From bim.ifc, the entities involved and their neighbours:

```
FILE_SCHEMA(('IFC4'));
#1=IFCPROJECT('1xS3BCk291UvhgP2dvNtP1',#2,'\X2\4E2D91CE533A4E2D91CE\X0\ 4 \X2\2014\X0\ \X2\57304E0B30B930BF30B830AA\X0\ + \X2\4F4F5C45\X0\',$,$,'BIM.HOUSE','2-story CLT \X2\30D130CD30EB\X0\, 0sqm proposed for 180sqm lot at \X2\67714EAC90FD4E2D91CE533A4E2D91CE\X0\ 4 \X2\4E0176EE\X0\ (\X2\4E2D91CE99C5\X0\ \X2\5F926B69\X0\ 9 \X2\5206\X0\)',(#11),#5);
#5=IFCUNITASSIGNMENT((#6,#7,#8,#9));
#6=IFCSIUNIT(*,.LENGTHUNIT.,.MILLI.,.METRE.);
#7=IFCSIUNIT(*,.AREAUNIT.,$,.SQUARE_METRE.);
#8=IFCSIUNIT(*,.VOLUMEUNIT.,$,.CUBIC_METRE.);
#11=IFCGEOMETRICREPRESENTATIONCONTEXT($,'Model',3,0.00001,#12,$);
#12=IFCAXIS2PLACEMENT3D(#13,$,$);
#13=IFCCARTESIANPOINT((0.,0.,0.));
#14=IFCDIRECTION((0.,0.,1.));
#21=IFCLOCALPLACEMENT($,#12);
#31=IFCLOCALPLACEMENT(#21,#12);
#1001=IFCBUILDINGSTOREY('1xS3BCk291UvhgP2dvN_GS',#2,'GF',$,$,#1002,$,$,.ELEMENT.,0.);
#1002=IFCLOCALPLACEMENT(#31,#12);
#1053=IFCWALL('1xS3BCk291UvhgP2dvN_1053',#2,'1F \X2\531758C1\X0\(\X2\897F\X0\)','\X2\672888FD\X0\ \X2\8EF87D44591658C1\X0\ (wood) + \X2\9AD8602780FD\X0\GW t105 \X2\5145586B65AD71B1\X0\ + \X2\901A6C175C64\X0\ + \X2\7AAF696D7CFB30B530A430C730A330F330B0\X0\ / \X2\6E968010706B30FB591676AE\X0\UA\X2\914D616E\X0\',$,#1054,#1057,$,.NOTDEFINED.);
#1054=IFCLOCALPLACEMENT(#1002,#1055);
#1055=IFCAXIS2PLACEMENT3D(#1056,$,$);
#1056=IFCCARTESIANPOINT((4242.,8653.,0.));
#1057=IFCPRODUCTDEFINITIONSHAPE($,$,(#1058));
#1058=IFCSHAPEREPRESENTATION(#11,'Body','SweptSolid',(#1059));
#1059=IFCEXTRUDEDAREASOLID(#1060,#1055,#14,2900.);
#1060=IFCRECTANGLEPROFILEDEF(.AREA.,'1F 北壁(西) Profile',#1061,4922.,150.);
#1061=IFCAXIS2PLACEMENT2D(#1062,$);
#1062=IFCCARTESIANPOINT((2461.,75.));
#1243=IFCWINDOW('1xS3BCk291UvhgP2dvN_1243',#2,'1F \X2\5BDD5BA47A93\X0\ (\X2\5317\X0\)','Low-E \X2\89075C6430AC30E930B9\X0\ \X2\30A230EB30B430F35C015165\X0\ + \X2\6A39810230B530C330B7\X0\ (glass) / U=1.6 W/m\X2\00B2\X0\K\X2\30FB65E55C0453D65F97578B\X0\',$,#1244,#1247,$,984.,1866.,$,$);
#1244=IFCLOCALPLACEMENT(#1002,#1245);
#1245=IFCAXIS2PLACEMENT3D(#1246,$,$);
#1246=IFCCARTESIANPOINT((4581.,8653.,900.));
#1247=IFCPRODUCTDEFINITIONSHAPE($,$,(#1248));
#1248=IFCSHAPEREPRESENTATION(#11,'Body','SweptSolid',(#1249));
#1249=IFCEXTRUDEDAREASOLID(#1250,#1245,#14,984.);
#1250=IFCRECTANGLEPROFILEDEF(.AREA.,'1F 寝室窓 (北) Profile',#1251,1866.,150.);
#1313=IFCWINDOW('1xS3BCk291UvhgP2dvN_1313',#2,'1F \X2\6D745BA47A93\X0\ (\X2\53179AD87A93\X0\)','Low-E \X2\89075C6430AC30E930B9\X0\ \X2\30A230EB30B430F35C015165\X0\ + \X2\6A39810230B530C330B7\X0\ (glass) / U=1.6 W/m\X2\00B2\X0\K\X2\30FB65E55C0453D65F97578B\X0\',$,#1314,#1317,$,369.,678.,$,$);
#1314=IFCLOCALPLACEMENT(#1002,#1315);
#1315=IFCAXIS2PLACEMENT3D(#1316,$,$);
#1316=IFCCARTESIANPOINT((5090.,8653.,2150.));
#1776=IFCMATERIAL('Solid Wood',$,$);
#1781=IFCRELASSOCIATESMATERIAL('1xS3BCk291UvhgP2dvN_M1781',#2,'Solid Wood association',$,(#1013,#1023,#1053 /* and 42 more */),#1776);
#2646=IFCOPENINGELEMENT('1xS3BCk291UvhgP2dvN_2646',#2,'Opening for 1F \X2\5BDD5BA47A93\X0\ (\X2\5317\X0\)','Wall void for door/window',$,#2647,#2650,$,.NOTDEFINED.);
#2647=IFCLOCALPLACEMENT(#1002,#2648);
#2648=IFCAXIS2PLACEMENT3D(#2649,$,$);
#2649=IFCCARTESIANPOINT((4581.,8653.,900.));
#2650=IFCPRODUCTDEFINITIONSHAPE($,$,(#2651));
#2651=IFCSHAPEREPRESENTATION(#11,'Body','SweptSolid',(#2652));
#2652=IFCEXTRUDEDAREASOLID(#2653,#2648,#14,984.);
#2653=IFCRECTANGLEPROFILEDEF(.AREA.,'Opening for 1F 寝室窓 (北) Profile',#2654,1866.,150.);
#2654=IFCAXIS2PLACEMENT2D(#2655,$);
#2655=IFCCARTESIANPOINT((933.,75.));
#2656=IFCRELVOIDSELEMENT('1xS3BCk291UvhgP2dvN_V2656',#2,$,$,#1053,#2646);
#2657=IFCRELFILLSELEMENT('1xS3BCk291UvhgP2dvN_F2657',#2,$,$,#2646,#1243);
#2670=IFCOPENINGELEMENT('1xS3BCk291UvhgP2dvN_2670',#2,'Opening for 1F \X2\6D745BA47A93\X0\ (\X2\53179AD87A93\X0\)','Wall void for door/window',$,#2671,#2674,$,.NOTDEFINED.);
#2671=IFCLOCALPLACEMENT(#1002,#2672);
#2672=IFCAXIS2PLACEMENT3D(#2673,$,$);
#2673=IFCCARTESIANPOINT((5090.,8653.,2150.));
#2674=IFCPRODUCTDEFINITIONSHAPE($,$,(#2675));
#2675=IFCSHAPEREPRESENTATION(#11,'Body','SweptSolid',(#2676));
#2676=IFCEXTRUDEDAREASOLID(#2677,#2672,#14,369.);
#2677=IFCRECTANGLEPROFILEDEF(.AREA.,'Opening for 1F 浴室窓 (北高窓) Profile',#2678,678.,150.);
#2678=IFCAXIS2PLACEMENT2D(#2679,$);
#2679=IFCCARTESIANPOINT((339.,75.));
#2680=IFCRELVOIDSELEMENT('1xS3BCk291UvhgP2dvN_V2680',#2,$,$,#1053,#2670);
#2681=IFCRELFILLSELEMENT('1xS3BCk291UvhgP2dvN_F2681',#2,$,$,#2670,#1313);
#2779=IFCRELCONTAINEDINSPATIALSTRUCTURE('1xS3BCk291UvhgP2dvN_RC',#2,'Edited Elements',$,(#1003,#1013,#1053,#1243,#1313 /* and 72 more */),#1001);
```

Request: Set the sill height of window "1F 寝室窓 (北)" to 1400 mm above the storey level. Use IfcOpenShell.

```python
import numpy as np
import ifcopenshell
import ifcopenshell.api.geometry
import ifcopenshell.geom
import ifcopenshell.util.element
import ifcopenshell.util.placement
import ifcopenshell.util.shape
import ifcopenshell.util.unit

model = ifcopenshell.open("bim.ifc")
unit_scale = ifcopenshell.util.unit.calculate_unit_scale(model)

window = model.by_guid("1xS3BCk291UvhgP2dvN_1243")
opening = window.FillsVoids[0].RelatingOpeningElement
storey = ifcopenshell.util.element.get_container(window, ifc_class="IfcBuildingStorey")
level = ifcopenshell.util.placement.get_local_placement(storey.ObjectPlacement)[2, 3]

# The opening's origin need not be at the sill, so measure its lowest point.
shape = ifcopenshell.geom.create_shape(ifcopenshell.geom.settings(), opening)
bottom = ifcopenshell.util.shape.get_shape_bottom_elevation(shape, shape.geometry) / unit_scale
dz = level + 1.4 / unit_scale - bottom

shift = np.array([0.0, 0.0, dz])
# The window is not placed relative to its opening, so move both.
for product in (opening, window):
    matrix = ifcopenshell.util.placement.get_local_placement(product.ObjectPlacement)
    matrix[:3, 3] += shift
    ifcopenshell.api.geometry.edit_object_placement(model, product=product, matrix=matrix, is_si=False)

print(f"moved by {dz * unit_scale:+.3f} m")

model.write("bim_updated.ifc")
```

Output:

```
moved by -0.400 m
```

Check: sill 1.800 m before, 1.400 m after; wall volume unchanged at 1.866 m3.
